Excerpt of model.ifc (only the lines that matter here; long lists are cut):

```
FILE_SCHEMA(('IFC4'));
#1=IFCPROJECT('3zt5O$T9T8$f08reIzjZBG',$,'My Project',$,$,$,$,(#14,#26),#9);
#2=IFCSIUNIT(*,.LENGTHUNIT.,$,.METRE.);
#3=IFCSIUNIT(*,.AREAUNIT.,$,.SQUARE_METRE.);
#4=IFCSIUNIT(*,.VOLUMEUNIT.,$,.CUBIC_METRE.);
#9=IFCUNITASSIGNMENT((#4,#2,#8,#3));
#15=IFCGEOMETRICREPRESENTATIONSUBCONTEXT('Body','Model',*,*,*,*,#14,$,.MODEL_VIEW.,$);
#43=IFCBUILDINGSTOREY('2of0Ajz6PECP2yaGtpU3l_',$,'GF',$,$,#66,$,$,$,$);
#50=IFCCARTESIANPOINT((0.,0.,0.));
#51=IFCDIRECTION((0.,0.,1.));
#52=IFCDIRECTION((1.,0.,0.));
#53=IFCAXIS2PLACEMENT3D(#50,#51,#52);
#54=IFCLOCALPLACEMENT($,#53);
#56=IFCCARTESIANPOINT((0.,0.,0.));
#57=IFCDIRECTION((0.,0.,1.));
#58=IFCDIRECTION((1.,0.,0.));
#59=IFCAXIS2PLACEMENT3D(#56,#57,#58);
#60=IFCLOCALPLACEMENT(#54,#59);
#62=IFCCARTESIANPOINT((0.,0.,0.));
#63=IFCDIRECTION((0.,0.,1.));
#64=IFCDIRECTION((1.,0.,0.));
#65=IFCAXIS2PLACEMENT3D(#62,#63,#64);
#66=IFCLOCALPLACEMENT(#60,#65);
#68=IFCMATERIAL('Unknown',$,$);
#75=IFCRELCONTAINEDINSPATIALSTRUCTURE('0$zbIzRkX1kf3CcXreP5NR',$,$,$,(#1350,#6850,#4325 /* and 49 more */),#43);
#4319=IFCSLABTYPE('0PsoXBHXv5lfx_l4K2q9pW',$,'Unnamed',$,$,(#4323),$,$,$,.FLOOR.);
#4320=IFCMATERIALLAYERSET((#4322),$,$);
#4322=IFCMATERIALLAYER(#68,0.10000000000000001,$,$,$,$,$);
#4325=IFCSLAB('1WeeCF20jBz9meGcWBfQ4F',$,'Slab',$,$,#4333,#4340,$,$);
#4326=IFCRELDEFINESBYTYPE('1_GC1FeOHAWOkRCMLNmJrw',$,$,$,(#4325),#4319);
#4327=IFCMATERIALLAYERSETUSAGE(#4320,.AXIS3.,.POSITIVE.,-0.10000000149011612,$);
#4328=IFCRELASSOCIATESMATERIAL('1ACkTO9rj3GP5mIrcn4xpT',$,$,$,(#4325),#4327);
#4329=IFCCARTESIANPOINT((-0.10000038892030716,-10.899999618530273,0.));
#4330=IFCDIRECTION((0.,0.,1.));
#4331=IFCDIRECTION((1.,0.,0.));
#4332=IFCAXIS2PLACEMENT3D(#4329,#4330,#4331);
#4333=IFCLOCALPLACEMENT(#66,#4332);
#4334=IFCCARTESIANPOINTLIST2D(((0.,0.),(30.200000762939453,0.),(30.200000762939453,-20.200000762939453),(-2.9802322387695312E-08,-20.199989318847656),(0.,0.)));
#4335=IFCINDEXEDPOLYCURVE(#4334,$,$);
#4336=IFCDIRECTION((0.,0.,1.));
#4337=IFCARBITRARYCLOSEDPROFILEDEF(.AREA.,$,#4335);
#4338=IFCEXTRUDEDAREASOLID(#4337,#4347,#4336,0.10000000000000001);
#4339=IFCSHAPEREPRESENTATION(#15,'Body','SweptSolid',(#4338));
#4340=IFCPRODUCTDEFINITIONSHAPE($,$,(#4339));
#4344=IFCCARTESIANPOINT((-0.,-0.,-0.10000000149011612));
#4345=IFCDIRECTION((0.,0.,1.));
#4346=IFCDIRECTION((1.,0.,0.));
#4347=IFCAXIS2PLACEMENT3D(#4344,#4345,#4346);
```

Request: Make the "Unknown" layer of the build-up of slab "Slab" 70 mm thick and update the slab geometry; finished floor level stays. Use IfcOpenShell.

```python
import ifcopenshell
import ifcopenshell.util.element
import ifcopenshell.util.representation

model = ifcopenshell.open("model.ifc")

layer_set = model.by_id(4320)
layer = next(l for l in layer_set.MaterialLayers if l.Material and l.Material.Name == "Unknown")
change = 0.07 - layer.LayerThickness
layer.LayerThickness += change

# Geometry does not follow the layer set by itself.
slabs = [e for e in ifcopenshell.util.element.get_elements_by_material(model, layer_set) if e.is_a("IfcSlab")]
for slab in sorted(slabs, key=lambda e: e.id()):
    body = ifcopenshell.util.representation.get_representation(slab, "Model", "Body")
    solid = body.Items[0]
    old_depth = solid.Depth
    solid.Depth += change
    # Extruded upwards: lower the start of the extrusion so the top stays.
    x, y, z = solid.Position.Location.Coordinates
    solid.Position.Location = model.createIfcCartesianPoint((x, y, z - change))
    print(slab.id(), f"{old_depth:g} -> {solid.Depth:g}")

# The layers are counted up from the underside, which has moved.
for usage in {ifcopenshell.util.element.get_material(slab) for slab in slabs}:
    usage.OffsetFromReferenceLine -= change

model.write("model_edited.ifc")
```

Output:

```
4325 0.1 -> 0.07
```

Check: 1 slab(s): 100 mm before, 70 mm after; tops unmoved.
